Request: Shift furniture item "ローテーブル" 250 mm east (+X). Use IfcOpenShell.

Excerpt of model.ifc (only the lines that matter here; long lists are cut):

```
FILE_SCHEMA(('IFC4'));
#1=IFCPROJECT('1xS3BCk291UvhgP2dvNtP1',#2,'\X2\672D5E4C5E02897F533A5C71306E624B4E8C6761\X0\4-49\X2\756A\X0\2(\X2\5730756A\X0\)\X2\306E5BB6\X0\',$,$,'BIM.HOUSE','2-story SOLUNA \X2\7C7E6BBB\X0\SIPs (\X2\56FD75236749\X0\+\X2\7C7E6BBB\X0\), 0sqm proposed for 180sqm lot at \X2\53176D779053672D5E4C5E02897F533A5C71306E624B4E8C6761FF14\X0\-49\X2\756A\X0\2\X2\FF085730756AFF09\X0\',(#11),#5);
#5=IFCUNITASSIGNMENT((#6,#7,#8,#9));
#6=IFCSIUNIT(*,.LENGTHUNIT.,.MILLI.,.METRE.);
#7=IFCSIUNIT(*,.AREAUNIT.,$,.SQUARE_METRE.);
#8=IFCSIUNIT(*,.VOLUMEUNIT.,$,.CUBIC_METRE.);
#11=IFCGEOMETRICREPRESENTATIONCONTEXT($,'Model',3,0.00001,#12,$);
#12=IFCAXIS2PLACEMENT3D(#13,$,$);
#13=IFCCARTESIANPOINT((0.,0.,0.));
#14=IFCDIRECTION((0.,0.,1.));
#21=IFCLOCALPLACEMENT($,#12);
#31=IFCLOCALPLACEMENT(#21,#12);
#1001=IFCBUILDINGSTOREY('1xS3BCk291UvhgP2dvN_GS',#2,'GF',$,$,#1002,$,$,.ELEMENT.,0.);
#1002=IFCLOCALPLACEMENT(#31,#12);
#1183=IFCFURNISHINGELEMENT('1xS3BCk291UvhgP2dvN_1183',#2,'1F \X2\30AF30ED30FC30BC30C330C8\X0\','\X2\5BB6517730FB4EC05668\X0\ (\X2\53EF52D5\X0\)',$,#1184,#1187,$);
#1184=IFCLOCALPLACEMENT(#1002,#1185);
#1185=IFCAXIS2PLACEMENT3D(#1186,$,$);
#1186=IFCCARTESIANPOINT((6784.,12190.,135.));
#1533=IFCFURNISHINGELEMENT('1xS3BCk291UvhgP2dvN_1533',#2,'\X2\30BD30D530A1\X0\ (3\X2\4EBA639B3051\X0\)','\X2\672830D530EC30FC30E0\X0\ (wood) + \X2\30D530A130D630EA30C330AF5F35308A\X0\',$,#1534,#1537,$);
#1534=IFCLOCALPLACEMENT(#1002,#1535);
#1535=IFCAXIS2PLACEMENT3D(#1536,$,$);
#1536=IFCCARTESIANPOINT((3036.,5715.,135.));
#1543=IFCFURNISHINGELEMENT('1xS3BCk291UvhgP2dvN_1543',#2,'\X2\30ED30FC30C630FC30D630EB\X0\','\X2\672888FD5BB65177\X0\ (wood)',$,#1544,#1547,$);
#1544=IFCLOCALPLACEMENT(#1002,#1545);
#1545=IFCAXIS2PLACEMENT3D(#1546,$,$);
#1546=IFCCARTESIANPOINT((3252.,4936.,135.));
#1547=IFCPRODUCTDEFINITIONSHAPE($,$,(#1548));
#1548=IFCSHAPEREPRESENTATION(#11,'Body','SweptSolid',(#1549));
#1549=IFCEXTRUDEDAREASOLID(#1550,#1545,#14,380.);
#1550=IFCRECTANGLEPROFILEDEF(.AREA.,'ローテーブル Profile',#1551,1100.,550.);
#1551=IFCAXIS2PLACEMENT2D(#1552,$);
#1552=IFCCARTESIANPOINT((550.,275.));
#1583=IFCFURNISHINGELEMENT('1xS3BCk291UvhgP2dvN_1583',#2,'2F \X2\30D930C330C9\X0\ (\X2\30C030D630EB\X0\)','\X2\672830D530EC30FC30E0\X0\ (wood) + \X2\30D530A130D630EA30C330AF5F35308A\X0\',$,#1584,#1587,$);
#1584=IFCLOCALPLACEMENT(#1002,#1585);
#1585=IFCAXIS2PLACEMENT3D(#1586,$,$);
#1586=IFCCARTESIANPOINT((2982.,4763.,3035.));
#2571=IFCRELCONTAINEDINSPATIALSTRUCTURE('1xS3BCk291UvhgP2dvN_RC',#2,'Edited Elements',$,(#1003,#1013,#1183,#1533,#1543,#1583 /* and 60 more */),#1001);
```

```python
import ifcopenshell
import ifcopenshell.api.geometry
import ifcopenshell.util.placement

model = ifcopenshell.open("model.ifc")

item = model.by_guid("1xS3BCk291UvhgP2dvN_1543")
matrix = ifcopenshell.util.placement.get_local_placement(item.ObjectPlacement)
matrix[0, 3] += 250.0
ifcopenshell.api.geometry.edit_object_placement(model, product=item, matrix=matrix, is_si=False)

print(ifcopenshell.util.placement.get_local_placement(item.ObjectPlacement).round(3) + 0.0)

model.write("model_v2.ifc")
```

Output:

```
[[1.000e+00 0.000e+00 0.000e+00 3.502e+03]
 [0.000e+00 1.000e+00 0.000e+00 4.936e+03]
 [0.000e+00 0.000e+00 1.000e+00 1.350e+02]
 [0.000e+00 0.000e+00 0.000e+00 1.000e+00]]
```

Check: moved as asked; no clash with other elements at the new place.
